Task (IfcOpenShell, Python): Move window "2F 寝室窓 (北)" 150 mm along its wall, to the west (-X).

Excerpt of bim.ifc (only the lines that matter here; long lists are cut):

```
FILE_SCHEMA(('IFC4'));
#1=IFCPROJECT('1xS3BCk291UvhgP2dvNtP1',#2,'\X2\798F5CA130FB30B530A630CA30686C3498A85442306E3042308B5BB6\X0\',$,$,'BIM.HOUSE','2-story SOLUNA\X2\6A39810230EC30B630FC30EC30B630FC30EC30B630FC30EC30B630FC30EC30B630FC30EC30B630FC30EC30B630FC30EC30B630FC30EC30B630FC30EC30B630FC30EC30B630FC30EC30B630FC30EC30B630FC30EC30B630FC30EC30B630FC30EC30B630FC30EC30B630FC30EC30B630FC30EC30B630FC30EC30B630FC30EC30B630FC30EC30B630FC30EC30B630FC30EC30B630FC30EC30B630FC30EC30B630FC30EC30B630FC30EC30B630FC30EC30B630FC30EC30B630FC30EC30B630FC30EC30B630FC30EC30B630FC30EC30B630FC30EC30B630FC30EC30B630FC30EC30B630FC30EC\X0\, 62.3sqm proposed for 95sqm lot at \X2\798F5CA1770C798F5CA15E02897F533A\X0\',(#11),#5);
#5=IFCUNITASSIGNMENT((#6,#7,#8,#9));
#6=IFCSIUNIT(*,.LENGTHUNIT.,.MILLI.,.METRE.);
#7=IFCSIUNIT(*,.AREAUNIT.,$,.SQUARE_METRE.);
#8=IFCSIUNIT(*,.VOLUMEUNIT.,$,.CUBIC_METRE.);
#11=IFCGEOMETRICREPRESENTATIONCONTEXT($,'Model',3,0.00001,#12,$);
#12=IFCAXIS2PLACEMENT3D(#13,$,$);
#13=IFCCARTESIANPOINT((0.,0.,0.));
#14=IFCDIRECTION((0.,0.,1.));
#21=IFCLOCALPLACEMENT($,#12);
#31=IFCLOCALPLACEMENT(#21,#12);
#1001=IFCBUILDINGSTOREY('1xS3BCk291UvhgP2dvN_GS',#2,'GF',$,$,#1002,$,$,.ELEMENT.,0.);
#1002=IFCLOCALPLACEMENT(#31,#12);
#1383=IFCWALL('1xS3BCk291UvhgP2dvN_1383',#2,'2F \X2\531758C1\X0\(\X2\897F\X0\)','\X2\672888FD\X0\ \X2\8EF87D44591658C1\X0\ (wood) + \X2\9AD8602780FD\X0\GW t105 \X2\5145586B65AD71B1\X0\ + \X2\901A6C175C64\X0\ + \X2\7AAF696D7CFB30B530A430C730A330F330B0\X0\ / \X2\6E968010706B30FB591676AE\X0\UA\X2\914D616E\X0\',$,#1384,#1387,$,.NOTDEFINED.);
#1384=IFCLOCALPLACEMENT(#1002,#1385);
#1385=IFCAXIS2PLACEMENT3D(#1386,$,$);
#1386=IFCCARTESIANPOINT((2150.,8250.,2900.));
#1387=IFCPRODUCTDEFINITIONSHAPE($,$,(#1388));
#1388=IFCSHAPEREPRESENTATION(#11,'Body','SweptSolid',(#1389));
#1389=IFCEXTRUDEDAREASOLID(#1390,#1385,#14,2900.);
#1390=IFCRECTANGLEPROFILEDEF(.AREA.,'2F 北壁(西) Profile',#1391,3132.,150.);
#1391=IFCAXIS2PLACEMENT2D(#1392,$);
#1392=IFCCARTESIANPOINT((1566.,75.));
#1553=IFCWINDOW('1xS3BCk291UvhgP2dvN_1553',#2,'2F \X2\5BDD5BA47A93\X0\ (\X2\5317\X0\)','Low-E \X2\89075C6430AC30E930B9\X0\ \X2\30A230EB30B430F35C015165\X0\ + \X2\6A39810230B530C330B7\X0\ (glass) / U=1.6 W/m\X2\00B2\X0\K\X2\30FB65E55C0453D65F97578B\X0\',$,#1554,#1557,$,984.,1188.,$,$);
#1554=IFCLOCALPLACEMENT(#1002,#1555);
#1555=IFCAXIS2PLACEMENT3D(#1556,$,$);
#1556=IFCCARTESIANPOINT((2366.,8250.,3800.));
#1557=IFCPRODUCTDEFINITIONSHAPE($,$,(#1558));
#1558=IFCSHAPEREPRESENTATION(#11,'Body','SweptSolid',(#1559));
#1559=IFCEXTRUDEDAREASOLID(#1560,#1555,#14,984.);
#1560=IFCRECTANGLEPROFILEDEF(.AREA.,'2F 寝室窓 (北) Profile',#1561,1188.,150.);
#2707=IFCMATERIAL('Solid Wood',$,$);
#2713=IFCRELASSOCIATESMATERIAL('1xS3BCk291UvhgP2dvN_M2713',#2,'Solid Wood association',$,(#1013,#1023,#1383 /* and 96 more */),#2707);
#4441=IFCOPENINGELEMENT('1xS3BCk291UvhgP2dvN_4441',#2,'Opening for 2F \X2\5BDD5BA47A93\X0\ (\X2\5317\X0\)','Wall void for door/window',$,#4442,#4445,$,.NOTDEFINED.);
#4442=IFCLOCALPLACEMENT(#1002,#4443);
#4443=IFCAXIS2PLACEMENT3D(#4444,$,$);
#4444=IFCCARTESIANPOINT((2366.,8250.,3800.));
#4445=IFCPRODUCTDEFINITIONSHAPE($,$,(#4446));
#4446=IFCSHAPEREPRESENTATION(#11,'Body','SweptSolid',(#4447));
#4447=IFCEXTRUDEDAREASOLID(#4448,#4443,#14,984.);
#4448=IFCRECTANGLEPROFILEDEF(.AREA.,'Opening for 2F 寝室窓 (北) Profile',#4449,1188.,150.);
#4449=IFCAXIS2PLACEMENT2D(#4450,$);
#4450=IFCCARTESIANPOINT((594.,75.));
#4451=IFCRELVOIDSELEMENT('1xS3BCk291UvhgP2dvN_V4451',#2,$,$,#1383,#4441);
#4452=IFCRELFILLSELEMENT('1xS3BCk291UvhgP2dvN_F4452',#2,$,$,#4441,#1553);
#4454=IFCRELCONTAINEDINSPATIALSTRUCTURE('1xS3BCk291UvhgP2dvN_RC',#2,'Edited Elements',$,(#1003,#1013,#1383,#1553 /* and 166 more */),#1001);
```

```python
import ifcopenshell
import ifcopenshell.api.geometry
import ifcopenshell.util.placement

model = ifcopenshell.open("bim.ifc")

window = model.by_guid("1xS3BCk291UvhgP2dvN_1553")
opening = window.FillsVoids[0].RelatingOpeningElement
wall = opening.VoidsElements[0].RelatingBuildingElement

wall_matrix = ifcopenshell.util.placement.get_local_placement(wall.ObjectPlacement)
shift = wall_matrix[:3, 0] * -150.0
before = ifcopenshell.util.placement.get_local_placement(window.ObjectPlacement)[:3, 3].copy()

# The window is not placed relative to its opening, so move both.
for product in (opening, window):
    matrix = ifcopenshell.util.placement.get_local_placement(product.ObjectPlacement)
    matrix[:3, 3] += shift
    ifcopenshell.api.geometry.edit_object_placement(model, product=product, matrix=matrix, is_si=False)

after = ifcopenshell.util.placement.get_local_placement(window.ObjectPlacement)[:3, 3]
print("window moved by", (after - before).round(3) + 0.0)

model.write("bim_updated.ifc")
```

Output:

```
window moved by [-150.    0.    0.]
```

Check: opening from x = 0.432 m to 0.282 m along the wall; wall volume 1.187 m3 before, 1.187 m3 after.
